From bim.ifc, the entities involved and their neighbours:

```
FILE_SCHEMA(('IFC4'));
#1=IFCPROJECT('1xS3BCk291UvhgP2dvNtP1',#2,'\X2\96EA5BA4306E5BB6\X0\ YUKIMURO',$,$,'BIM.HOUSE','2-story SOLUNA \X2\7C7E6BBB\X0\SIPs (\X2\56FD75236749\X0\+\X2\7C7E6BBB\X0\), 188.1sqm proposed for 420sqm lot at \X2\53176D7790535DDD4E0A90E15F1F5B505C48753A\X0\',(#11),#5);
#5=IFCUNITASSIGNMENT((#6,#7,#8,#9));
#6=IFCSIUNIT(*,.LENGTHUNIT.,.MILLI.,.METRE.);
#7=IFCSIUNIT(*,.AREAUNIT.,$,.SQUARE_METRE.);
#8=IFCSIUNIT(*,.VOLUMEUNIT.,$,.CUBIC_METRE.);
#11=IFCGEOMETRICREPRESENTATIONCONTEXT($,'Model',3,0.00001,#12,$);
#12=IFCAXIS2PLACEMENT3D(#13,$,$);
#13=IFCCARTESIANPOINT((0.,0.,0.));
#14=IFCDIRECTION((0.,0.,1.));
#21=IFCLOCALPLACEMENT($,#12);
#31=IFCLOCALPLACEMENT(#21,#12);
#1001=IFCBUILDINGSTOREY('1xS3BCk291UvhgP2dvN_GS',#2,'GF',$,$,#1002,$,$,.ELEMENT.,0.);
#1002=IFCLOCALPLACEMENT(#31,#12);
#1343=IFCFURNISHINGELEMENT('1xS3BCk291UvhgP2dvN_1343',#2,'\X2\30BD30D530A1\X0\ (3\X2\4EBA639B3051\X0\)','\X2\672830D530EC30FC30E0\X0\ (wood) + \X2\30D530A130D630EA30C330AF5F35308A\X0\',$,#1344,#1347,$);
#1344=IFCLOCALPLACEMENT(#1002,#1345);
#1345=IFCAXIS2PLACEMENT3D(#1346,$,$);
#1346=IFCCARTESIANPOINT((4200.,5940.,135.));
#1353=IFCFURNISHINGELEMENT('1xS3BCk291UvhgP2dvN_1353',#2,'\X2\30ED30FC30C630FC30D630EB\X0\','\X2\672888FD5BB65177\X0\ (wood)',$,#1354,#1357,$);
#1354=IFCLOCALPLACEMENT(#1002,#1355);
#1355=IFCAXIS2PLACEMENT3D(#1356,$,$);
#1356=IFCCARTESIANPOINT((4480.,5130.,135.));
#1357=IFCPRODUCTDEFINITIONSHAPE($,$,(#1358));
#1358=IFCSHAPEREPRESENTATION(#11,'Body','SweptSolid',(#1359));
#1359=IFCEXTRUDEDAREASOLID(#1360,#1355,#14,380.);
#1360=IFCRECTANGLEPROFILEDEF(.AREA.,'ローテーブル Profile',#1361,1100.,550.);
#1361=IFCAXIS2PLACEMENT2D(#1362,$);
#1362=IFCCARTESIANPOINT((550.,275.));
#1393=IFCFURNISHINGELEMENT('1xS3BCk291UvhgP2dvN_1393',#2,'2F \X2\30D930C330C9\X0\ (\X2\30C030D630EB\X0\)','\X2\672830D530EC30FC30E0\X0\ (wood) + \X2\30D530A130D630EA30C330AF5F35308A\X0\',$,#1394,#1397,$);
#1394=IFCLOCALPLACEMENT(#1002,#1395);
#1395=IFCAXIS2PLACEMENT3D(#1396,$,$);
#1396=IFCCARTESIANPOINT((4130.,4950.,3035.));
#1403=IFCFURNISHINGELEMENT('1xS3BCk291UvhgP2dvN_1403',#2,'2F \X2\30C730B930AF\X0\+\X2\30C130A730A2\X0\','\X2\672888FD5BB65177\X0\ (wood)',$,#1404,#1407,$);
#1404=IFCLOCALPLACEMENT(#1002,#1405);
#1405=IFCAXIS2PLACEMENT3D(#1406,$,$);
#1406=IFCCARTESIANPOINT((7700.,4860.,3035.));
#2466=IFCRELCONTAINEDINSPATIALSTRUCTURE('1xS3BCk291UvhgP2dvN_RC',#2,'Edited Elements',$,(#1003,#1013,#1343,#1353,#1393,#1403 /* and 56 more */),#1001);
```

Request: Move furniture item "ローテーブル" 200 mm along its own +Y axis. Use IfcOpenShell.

```python
import ifcopenshell
import ifcopenshell.api.geometry
import ifcopenshell.util.placement
import ifcopenshell.util.unit

model = ifcopenshell.open("bim.ifc")
unit_scale = ifcopenshell.util.unit.calculate_unit_scale(model)

item = model.by_id(1353)
matrix = ifcopenshell.util.placement.get_local_placement(item.ObjectPlacement)
matrix[:3, 3] += matrix[:3, 1] * 0.2 / unit_scale
ifcopenshell.api.geometry.edit_object_placement(model, product=item, matrix=matrix, is_si=False)

print(ifcopenshell.util.placement.get_local_placement(item.ObjectPlacement).round(3) + 0.0)

model.write("bim_edited.ifc")
```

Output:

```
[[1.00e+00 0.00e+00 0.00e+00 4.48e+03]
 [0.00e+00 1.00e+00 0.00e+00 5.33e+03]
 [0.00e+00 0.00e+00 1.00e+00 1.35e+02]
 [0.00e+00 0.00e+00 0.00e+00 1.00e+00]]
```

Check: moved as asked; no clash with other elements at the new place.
